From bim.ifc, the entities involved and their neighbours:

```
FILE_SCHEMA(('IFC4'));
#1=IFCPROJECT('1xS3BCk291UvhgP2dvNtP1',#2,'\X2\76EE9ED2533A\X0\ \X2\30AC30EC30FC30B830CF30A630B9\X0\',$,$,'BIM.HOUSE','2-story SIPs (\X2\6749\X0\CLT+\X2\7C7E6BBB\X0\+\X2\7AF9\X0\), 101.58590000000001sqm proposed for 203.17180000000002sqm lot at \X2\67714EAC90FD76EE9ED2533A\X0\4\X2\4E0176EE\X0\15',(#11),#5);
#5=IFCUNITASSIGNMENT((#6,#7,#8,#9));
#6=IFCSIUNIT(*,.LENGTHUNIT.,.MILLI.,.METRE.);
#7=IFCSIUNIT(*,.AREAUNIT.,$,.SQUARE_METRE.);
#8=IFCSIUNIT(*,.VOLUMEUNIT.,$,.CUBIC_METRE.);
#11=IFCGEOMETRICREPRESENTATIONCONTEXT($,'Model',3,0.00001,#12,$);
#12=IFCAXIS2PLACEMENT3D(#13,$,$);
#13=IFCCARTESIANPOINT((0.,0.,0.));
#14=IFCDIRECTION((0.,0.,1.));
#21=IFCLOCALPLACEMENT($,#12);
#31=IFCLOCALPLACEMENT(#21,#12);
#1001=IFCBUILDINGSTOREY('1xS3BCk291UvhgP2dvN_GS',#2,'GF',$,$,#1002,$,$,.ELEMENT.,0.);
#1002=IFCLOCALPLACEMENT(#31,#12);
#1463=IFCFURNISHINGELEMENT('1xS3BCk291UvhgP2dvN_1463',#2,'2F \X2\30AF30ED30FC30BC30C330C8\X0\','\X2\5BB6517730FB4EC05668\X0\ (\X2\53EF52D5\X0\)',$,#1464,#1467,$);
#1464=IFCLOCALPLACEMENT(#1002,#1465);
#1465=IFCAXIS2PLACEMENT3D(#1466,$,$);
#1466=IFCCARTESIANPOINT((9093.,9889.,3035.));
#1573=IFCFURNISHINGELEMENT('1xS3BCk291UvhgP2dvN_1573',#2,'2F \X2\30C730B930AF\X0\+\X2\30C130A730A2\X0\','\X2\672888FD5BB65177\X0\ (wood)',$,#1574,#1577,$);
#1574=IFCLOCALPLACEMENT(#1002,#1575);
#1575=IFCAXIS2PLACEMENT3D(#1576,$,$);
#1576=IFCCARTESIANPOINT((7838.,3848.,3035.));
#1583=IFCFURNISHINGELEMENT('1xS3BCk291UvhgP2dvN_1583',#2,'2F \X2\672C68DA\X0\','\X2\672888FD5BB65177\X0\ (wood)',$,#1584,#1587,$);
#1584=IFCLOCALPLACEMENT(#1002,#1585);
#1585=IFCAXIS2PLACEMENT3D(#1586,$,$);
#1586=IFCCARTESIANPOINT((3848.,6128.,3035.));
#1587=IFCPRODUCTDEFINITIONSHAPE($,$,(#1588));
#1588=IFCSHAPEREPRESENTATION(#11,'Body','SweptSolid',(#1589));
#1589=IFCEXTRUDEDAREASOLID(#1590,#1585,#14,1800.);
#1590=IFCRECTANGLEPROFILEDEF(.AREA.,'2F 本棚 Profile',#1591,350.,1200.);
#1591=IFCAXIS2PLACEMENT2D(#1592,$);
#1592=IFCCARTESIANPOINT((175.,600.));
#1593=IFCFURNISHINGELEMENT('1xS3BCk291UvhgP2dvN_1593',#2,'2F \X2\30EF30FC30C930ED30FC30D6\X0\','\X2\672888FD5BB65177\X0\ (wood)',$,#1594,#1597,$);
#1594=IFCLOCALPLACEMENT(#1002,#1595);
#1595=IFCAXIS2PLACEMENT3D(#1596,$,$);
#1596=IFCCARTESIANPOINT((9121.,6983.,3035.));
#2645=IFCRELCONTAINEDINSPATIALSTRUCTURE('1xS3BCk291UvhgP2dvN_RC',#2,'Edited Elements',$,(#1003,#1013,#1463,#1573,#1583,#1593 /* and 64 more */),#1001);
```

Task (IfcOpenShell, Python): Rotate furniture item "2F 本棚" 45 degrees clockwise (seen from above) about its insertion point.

```python
import ifcopenshell
import ifcopenshell.api.geometry
import ifcopenshell.util.placement

model = ifcopenshell.open("bim.ifc")

item = model.by_guid("1xS3BCk291UvhgP2dvN_1583")
matrix = ifcopenshell.util.placement.get_local_placement(item.ObjectPlacement)
matrix = matrix @ ifcopenshell.util.placement.rotation(-45, "Z")
ifcopenshell.api.geometry.edit_object_placement(model, product=item, matrix=matrix, is_si=False)

print(ifcopenshell.util.placement.get_local_placement(item.ObjectPlacement).round(3) + 0.0)

model.write("bim_edited.ifc")
```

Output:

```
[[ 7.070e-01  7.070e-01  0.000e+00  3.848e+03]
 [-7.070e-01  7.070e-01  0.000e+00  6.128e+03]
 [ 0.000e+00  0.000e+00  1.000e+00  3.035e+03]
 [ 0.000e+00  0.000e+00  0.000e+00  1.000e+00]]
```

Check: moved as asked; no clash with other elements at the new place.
